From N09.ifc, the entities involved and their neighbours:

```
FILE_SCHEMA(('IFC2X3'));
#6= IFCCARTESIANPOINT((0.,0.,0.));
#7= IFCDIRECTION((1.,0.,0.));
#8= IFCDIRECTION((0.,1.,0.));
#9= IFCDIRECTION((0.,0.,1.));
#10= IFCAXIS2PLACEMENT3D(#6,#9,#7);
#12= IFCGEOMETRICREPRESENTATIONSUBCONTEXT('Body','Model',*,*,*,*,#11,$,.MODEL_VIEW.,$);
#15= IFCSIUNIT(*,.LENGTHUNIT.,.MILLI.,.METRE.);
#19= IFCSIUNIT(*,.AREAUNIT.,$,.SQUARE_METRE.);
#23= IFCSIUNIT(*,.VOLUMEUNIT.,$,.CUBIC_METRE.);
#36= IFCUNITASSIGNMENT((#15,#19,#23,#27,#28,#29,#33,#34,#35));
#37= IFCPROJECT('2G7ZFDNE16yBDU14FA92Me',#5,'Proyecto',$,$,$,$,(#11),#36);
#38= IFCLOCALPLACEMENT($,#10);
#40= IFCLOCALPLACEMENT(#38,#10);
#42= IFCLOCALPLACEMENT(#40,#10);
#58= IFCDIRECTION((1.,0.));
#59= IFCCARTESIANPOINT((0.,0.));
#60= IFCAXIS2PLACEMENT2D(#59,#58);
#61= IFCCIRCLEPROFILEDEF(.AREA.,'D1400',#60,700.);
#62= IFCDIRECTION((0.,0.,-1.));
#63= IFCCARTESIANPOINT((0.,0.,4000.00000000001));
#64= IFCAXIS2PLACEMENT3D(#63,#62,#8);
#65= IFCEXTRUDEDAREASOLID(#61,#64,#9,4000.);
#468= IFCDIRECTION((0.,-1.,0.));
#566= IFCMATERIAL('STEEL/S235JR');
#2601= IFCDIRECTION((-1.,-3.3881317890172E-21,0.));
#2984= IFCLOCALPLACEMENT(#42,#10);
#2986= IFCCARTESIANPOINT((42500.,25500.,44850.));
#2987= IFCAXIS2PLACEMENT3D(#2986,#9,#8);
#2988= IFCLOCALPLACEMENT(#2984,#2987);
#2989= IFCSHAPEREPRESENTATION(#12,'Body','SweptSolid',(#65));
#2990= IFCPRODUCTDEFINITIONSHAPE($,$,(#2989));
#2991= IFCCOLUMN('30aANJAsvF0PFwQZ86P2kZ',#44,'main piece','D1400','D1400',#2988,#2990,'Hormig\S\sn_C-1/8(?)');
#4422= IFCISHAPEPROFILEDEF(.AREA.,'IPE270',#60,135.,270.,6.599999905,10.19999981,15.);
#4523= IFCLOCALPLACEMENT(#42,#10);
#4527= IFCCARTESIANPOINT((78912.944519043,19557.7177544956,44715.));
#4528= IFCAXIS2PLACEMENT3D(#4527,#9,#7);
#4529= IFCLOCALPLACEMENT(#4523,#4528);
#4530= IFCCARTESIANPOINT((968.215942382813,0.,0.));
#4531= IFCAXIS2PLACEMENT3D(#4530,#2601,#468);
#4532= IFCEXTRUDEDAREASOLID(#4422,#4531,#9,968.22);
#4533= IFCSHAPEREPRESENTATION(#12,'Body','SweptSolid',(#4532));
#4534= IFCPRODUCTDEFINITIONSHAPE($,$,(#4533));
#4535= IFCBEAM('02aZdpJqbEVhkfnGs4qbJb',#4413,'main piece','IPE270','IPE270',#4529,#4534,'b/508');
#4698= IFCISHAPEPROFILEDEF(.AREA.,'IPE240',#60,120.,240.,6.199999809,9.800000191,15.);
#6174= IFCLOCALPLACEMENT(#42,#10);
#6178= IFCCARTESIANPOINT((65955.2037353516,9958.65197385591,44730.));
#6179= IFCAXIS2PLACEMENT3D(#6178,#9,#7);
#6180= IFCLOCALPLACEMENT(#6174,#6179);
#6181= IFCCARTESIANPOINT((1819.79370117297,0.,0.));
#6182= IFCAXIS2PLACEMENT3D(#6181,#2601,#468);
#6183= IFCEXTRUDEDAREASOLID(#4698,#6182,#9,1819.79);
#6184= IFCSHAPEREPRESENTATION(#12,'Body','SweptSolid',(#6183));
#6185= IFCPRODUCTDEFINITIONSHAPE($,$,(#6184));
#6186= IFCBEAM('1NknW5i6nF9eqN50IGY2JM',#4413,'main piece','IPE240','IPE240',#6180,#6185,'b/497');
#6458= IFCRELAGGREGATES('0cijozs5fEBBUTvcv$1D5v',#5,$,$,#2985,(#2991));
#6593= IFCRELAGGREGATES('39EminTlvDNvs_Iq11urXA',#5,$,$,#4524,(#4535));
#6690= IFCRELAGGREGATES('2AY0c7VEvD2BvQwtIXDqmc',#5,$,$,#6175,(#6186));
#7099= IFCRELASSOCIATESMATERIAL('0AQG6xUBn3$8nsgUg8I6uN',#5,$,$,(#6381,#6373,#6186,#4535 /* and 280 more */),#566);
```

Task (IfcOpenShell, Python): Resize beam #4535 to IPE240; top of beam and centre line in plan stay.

```python
import ifcopenshell
import ifcopenshell.util.element
import ifcopenshell.util.representation

model = ifcopenshell.open("N09.ifc")

member = model.by_id(4535)
source = next(p for p in model.by_type("IfcIShapeProfileDef") if p.ProfileName == "IPE240")

body = ifcopenshell.util.representation.get_representation(member, "Model", "Body")
solid = body.Items[0]
old_profile = solid.SweptArea

# Copy the section's sizes but keep this member's own profile position.
profile = ifcopenshell.util.element.copy(model, source)
# Profiles are centred, so shift by half the change in depth to hold the top.
shift = (old_profile.OverallDepth - profile.OverallDepth) / 2
x, y = old_profile.Position.Location.Coordinates
up = (0.0, 1.0)  # upwards, in the solid's own plane
location = model.createIfcCartesianPoint((x + up[0] * shift, y + up[1] * shift))
profile.Position = model.createIfcAxis2Placement2D(location, old_profile.Position.RefDirection)
solid.SweptArea = profile
if not model.get_total_inverses(old_profile):
    ifcopenshell.util.element.remove_deep2(model, old_profile)
member.Description = member.Description.replace("IPE270", "IPE240")
member.ObjectType = member.ObjectType.replace("IPE270", "IPE240")

print(solid.SweptArea)

model.write("N09_updated.ifc")
```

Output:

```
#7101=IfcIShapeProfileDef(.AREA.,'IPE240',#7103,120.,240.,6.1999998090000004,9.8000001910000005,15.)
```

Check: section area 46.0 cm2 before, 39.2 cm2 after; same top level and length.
